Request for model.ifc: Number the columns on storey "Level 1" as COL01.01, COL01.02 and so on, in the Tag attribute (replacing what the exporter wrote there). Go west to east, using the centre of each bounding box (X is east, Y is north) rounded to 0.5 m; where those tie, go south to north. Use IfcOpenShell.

First a look at what the model holds.

```python
import ifcopenshell
import ifcopenshell.util.element
import ifcopenshell.util.placement

model = ifcopenshell.open("model.ifc")
print(model.schema)
storey = next(s for s in model.by_type("IfcBuildingStorey") if s.Name == "Level 1")
columns = [e for e in ifcopenshell.util.element.get_decomposition(storey) if e.is_a("IfcColumn")]
for e in sorted(columns, key=lambda e: e.id()):
    origin = ifcopenshell.util.placement.get_local_placement(e.ObjectPlacement)[:3, 3]
    print(e.id(), e.Tag, e.Name, origin.round(2) + 0.0, sep=" | ")
```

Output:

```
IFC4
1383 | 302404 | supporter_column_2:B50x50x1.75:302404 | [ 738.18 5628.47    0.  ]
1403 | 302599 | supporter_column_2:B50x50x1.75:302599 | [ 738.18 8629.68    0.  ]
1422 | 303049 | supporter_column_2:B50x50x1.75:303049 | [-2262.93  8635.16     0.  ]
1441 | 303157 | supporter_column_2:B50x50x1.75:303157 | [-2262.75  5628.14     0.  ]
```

```python
import ifcopenshell
import ifcopenshell.geom
import ifcopenshell.util.element
import ifcopenshell.util.shape

model = ifcopenshell.open("model.ifc")
settings = ifcopenshell.geom.settings()
settings.set("use-world-coords", True)


def centre(element):
    shape = ifcopenshell.geom.create_shape(settings, element)
    return ifcopenshell.util.shape.get_bbox_centroid(shape.geometry)


storey = next(s for s in model.by_type("IfcBuildingStorey") if s.Name == "Level 1")
columns = [e for e in ifcopenshell.util.element.get_decomposition(storey) if e.is_a("IfcColumn")]

# Insertion points can sit at a corner or the storey origin, so sort by the geometry (in metres).
centres = {e: centre(e) for e in columns}
columns.sort(key=lambda e: (round(centres[e][0] / 0.5), centres[e][1]))

for i, e in enumerate(columns, start=1):
    number = f"COL01.{i:02d}"
    e.Tag = number
    print(e.id(), number)

model.write("model_updated.ifc")
```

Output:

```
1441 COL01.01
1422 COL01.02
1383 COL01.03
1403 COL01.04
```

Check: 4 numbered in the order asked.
